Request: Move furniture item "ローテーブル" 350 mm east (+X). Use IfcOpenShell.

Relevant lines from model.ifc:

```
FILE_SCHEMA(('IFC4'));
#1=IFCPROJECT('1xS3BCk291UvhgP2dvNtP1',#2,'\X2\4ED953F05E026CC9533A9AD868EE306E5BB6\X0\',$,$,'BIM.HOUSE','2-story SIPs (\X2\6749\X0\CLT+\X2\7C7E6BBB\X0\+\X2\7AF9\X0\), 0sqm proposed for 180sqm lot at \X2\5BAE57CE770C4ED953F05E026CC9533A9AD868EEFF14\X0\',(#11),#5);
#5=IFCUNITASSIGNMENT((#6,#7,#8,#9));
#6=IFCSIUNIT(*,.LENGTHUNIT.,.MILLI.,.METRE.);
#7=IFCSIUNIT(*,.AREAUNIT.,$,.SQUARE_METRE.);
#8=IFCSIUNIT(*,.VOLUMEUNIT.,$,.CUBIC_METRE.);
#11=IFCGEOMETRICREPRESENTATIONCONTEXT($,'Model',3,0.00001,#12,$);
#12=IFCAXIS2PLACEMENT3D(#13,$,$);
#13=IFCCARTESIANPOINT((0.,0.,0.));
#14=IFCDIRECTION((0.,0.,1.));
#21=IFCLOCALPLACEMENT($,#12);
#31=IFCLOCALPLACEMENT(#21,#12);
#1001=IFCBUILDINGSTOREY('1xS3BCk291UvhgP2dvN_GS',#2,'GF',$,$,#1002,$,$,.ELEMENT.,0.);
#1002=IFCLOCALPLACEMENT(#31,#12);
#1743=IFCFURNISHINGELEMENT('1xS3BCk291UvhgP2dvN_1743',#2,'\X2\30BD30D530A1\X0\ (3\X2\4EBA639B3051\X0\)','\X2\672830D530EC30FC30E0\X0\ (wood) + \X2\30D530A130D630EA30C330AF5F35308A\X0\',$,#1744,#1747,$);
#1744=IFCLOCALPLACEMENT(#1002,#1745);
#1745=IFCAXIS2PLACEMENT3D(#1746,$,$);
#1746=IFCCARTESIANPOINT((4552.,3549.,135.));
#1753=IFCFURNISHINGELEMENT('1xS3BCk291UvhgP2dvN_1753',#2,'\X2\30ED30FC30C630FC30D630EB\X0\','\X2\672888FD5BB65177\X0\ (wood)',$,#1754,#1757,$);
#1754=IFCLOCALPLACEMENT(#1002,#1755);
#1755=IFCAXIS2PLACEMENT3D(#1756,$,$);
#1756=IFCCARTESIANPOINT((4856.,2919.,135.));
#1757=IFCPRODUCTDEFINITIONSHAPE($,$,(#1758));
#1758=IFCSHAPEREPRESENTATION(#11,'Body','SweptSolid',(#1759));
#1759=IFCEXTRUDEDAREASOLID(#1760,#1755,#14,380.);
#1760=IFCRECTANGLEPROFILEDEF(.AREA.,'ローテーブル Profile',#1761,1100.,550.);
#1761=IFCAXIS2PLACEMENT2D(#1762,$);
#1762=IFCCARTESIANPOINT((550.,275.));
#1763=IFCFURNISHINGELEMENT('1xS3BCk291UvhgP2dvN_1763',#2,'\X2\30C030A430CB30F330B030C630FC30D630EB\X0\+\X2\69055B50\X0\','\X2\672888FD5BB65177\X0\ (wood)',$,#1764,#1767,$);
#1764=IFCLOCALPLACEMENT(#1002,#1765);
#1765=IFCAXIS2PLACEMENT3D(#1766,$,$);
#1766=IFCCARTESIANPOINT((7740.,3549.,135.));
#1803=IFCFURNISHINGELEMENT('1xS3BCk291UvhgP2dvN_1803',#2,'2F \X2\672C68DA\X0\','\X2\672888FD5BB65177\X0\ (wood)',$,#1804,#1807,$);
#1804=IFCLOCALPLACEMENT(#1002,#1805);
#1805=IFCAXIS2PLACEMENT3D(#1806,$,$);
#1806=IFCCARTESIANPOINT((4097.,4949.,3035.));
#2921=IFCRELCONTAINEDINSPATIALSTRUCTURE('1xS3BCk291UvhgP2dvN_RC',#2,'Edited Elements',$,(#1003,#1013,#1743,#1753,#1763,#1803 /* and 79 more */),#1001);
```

```python
import ifcopenshell
import ifcopenshell.api.geometry
import ifcopenshell.util.placement

model = ifcopenshell.open("model.ifc")

item = model.by_guid("1xS3BCk291UvhgP2dvN_1753")
matrix = ifcopenshell.util.placement.get_local_placement(item.ObjectPlacement)
matrix[0, 3] += 350.0
ifcopenshell.api.geometry.edit_object_placement(model, product=item, matrix=matrix, is_si=False)

print(ifcopenshell.util.placement.get_local_placement(item.ObjectPlacement).round(3) + 0.0)

model.write("model_v2.ifc")
```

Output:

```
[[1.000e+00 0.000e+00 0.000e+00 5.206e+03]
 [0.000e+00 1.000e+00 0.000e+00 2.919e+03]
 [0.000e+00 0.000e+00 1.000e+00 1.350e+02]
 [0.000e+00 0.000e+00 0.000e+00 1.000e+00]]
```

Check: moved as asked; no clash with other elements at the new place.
